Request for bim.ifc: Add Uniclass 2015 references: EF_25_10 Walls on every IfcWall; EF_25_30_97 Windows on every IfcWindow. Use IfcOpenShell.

First a look at what the model holds.

```python
import ifcopenshell

model = ifcopenshell.open("bim.ifc")
print(model.schema)
print("classifications:", [c.Name for c in model.by_type("IfcClassification")])
for ifc_class in ("IfcDoor", "IfcRoof", "IfcStair", "IfcWall", "IfcWindow"):
    print(ifc_class, len(model.by_type(ifc_class)))
```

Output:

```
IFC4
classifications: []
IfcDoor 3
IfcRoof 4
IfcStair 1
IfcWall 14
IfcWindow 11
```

```python
import ifcopenshell
import ifcopenshell.api.classification

model = ifcopenshell.open("bim.ifc")

system = ifcopenshell.api.classification.add_classification(model, classification="Uniclass 2015")

codes = {
    "IfcWall": ("EF_25_10", "Walls"),
    "IfcWindow": ("EF_25_30_97", "Windows"),
}
for ifc_class, (code, name) in codes.items():
    products = model.by_type(ifc_class)
    ifcopenshell.api.classification.add_reference(
        model, products=products, classification=system, identification=code, name=name
    )
    print(code, len(products))

model.write("bim_rev.ifc")
```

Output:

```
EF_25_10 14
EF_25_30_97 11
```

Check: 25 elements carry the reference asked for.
